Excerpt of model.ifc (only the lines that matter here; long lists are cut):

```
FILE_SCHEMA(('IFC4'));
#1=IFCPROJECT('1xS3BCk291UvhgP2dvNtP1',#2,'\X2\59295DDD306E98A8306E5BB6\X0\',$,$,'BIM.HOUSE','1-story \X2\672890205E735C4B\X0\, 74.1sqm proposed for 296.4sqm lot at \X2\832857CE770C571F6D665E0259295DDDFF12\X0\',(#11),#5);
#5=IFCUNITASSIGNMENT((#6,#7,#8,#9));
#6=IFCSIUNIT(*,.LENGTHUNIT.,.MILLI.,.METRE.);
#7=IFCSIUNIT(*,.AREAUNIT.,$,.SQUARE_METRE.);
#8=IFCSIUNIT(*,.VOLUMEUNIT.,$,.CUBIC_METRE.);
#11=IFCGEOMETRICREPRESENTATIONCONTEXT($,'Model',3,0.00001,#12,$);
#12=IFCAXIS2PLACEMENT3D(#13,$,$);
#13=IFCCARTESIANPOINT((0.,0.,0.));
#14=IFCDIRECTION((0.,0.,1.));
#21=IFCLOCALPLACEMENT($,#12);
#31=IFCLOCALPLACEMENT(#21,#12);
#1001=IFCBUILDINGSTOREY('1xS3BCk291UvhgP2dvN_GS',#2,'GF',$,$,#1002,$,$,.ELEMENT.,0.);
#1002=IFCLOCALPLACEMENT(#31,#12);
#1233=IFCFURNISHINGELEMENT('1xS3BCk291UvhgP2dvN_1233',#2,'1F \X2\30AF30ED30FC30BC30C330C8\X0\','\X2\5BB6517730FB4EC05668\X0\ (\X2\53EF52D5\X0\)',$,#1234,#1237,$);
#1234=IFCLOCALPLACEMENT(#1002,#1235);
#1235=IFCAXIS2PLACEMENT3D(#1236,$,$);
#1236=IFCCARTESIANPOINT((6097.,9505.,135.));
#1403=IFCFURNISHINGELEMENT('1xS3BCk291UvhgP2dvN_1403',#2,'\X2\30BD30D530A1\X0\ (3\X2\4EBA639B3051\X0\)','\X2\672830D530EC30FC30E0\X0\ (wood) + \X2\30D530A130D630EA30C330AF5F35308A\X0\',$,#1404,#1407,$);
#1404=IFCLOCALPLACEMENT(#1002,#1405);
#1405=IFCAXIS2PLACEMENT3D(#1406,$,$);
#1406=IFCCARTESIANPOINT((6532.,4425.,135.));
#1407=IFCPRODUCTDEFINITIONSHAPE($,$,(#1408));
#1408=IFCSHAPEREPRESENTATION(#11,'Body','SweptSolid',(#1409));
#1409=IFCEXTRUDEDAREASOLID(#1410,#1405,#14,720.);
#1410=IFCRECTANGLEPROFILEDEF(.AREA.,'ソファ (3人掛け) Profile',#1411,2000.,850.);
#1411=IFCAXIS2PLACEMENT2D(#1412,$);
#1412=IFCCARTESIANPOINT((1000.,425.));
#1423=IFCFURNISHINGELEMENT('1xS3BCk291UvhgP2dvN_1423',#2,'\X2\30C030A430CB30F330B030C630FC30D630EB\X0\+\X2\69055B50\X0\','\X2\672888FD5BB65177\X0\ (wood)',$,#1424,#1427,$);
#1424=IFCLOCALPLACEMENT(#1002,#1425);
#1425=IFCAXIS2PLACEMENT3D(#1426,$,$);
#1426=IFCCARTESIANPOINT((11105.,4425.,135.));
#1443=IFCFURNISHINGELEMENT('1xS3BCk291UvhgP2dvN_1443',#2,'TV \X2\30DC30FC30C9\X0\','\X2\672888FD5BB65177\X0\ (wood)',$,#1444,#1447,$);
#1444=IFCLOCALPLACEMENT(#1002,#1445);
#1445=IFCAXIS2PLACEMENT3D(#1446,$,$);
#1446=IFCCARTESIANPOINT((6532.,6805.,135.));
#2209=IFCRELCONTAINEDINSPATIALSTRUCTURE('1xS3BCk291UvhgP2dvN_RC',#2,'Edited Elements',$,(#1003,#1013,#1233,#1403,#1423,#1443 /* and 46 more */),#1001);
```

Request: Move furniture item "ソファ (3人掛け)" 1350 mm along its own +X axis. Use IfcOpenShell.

```python
import ifcopenshell
import ifcopenshell.api.geometry
import ifcopenshell.util.placement
import ifcopenshell.util.unit

model = ifcopenshell.open("model.ifc")
unit_scale = ifcopenshell.util.unit.calculate_unit_scale(model)

item = model.by_id(1403)
matrix = ifcopenshell.util.placement.get_local_placement(item.ObjectPlacement)
matrix[:3, 3] += matrix[:3, 0] * 1.35 / unit_scale
ifcopenshell.api.geometry.edit_object_placement(model, product=item, matrix=matrix, is_si=False)

print(ifcopenshell.util.placement.get_local_placement(item.ObjectPlacement).round(3) + 0.0)

model.write("model_rev.ifc")
```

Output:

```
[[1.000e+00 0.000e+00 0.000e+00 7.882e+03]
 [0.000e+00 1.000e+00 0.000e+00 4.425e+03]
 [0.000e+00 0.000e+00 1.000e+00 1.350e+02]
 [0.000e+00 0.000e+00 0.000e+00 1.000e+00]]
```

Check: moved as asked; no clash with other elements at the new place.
